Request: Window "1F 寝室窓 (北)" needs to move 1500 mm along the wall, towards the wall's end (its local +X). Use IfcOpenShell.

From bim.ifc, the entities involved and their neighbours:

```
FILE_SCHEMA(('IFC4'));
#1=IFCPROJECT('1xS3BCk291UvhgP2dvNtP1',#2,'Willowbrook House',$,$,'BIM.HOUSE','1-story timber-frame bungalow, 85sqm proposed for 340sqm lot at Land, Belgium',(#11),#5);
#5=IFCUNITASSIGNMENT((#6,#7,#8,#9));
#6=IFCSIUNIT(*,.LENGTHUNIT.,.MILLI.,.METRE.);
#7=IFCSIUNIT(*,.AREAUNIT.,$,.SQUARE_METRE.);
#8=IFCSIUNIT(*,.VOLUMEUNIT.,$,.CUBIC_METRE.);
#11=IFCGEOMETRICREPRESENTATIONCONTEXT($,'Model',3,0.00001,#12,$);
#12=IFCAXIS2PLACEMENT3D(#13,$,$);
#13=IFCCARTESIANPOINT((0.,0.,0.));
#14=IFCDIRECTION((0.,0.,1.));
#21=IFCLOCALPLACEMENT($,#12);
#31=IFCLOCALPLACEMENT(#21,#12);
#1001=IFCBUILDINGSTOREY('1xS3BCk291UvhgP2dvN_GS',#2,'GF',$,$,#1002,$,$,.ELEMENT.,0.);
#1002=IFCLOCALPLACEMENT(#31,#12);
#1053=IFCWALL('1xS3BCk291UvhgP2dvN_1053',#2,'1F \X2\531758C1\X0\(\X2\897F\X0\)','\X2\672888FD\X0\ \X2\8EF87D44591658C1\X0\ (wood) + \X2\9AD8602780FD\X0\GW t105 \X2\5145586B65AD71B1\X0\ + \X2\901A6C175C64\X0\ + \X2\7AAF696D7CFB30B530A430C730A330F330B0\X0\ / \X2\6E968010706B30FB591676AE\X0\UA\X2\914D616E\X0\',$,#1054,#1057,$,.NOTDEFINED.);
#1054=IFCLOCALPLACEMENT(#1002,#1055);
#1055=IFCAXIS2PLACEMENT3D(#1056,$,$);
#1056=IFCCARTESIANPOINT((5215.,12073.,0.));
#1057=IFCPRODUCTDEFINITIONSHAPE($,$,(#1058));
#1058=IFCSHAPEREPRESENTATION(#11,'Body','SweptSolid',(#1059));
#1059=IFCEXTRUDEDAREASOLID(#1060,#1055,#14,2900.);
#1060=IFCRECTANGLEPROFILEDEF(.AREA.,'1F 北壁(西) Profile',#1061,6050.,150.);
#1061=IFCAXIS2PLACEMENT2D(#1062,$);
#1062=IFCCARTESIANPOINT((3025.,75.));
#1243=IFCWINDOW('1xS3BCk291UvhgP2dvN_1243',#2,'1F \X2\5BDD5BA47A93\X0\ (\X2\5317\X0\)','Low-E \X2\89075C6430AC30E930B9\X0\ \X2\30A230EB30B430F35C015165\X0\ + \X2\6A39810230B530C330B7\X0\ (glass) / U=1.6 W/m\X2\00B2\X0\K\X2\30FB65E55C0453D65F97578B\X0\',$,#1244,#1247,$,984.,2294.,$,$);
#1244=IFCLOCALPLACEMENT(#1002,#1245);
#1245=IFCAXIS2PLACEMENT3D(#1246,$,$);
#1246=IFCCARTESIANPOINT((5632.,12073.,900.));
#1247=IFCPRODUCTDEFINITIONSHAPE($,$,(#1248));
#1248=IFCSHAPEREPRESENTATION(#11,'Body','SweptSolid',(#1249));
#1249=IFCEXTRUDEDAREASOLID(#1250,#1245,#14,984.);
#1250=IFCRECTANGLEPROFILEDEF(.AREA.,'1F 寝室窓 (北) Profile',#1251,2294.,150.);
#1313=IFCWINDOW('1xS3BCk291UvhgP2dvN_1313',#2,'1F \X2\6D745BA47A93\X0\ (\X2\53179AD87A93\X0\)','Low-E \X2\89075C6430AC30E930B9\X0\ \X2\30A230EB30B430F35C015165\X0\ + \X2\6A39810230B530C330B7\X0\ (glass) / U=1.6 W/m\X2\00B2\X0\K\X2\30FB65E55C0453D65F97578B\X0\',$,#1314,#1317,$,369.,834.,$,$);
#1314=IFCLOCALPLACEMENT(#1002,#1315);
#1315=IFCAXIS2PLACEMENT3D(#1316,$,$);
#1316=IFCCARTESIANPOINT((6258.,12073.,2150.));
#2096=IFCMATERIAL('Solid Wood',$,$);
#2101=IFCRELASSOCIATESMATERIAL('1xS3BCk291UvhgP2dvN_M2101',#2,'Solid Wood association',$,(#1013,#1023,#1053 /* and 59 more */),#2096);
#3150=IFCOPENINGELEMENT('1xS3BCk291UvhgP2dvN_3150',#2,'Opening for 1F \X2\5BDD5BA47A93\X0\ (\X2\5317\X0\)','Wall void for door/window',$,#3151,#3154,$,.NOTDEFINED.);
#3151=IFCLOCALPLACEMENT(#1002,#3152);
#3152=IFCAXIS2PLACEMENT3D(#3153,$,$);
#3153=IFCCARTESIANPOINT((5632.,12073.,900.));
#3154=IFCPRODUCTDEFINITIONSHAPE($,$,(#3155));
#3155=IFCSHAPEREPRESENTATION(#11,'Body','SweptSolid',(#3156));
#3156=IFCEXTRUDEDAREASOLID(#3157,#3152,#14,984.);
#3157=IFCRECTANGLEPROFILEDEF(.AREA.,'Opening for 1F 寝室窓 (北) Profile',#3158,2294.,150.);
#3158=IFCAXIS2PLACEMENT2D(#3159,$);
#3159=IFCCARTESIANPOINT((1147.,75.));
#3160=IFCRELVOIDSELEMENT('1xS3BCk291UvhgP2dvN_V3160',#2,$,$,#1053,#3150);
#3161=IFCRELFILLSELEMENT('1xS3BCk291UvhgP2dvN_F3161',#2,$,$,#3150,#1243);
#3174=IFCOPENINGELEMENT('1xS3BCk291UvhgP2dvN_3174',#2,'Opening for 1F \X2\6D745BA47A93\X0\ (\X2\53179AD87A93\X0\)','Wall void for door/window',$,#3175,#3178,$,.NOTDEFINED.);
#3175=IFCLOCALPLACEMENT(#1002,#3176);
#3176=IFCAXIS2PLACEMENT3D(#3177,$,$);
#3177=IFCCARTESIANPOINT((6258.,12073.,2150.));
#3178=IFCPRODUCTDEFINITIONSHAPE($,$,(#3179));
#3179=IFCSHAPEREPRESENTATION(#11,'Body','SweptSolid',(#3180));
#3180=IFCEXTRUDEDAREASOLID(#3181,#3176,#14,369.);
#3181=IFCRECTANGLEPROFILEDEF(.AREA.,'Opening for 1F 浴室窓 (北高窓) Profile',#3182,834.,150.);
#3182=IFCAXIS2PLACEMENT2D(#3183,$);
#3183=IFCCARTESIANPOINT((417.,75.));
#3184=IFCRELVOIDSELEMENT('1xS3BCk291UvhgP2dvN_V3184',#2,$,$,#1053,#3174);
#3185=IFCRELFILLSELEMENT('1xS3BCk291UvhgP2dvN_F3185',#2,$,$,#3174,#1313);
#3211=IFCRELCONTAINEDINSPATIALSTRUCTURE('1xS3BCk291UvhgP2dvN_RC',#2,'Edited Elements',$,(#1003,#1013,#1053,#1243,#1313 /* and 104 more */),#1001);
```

```python
import ifcopenshell
import ifcopenshell.api.geometry
import ifcopenshell.util.placement
import ifcopenshell.util.unit

model = ifcopenshell.open("bim.ifc")
unit_scale = ifcopenshell.util.unit.calculate_unit_scale(model)

window = model.by_guid("1xS3BCk291UvhgP2dvN_1243")
opening = window.FillsVoids[0].RelatingOpeningElement
wall = opening.VoidsElements[0].RelatingBuildingElement

wall_matrix = ifcopenshell.util.placement.get_local_placement(wall.ObjectPlacement)
shift = wall_matrix[:3, 0] * 1.5 / unit_scale
before = ifcopenshell.util.placement.get_local_placement(window.ObjectPlacement)[:3, 3].copy()

# The window is not placed relative to its opening, so move both.
for product in (opening, window):
    matrix = ifcopenshell.util.placement.get_local_placement(product.ObjectPlacement)
    matrix[:3, 3] += shift
    ifcopenshell.api.geometry.edit_object_placement(model, product=product, matrix=matrix, is_si=False)

after = ifcopenshell.util.placement.get_local_placement(window.ObjectPlacement)[:3, 3]
print("window moved by", (after - before).round(3) + 0.0)

model.write("bim_updated.ifc")
```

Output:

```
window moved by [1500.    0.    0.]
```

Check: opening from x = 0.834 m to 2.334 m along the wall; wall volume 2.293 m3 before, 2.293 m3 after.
